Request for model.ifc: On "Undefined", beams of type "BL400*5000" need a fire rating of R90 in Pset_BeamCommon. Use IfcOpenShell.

First a look at what the model holds.

```python
import ifcopenshell
import ifcopenshell.util.element

model = ifcopenshell.open("model.ifc")
print(model.schema)
storey = next(s for s in model.by_type("IfcBuildingStorey") if s.Name == "Undefined")
beams = [e for e in ifcopenshell.util.element.get_decomposition(storey) if e.is_a("IfcBeam")]
seen = {}
for e in beams:
    element_type = ifcopenshell.util.element.get_type(e)
    key = (element_type.Name if element_type != e and element_type else None, ifcopenshell.util.element.get_pset(e, "Pset_BeamCommon", "FireRating"))
    seen[key] = seen.get(key, 0) + 1
for (name, value), count in sorted(seen.items(), key=str):
    print(count, "x", name, "|", value)
```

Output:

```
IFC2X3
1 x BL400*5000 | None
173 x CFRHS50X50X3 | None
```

```python
import ifcopenshell
import ifcopenshell.api.pset
import ifcopenshell.util.element

model = ifcopenshell.open("model.ifc")

storey = next(s for s in model.by_type("IfcBuildingStorey") if s.Name == "Undefined")
beams = [e for e in ifcopenshell.util.element.get_decomposition(storey) if e.is_a("IfcBeam")]

count = 0
for e in beams:
    element_type = ifcopenshell.util.element.get_type(e)
    if element_type in (None, e) or element_type.Name != "BL400*5000":
        continue
    # add_pset returns the element's existing set when there is one.
    pset = ifcopenshell.api.pset.add_pset(model, product=e, name="Pset_BeamCommon")
    ifcopenshell.api.pset.edit_pset(model, pset=pset, properties={"FireRating": "R90"})
    count += 1

print(count, "beams updated")

model.write("model_updated.ifc")
```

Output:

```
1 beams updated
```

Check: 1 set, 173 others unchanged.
